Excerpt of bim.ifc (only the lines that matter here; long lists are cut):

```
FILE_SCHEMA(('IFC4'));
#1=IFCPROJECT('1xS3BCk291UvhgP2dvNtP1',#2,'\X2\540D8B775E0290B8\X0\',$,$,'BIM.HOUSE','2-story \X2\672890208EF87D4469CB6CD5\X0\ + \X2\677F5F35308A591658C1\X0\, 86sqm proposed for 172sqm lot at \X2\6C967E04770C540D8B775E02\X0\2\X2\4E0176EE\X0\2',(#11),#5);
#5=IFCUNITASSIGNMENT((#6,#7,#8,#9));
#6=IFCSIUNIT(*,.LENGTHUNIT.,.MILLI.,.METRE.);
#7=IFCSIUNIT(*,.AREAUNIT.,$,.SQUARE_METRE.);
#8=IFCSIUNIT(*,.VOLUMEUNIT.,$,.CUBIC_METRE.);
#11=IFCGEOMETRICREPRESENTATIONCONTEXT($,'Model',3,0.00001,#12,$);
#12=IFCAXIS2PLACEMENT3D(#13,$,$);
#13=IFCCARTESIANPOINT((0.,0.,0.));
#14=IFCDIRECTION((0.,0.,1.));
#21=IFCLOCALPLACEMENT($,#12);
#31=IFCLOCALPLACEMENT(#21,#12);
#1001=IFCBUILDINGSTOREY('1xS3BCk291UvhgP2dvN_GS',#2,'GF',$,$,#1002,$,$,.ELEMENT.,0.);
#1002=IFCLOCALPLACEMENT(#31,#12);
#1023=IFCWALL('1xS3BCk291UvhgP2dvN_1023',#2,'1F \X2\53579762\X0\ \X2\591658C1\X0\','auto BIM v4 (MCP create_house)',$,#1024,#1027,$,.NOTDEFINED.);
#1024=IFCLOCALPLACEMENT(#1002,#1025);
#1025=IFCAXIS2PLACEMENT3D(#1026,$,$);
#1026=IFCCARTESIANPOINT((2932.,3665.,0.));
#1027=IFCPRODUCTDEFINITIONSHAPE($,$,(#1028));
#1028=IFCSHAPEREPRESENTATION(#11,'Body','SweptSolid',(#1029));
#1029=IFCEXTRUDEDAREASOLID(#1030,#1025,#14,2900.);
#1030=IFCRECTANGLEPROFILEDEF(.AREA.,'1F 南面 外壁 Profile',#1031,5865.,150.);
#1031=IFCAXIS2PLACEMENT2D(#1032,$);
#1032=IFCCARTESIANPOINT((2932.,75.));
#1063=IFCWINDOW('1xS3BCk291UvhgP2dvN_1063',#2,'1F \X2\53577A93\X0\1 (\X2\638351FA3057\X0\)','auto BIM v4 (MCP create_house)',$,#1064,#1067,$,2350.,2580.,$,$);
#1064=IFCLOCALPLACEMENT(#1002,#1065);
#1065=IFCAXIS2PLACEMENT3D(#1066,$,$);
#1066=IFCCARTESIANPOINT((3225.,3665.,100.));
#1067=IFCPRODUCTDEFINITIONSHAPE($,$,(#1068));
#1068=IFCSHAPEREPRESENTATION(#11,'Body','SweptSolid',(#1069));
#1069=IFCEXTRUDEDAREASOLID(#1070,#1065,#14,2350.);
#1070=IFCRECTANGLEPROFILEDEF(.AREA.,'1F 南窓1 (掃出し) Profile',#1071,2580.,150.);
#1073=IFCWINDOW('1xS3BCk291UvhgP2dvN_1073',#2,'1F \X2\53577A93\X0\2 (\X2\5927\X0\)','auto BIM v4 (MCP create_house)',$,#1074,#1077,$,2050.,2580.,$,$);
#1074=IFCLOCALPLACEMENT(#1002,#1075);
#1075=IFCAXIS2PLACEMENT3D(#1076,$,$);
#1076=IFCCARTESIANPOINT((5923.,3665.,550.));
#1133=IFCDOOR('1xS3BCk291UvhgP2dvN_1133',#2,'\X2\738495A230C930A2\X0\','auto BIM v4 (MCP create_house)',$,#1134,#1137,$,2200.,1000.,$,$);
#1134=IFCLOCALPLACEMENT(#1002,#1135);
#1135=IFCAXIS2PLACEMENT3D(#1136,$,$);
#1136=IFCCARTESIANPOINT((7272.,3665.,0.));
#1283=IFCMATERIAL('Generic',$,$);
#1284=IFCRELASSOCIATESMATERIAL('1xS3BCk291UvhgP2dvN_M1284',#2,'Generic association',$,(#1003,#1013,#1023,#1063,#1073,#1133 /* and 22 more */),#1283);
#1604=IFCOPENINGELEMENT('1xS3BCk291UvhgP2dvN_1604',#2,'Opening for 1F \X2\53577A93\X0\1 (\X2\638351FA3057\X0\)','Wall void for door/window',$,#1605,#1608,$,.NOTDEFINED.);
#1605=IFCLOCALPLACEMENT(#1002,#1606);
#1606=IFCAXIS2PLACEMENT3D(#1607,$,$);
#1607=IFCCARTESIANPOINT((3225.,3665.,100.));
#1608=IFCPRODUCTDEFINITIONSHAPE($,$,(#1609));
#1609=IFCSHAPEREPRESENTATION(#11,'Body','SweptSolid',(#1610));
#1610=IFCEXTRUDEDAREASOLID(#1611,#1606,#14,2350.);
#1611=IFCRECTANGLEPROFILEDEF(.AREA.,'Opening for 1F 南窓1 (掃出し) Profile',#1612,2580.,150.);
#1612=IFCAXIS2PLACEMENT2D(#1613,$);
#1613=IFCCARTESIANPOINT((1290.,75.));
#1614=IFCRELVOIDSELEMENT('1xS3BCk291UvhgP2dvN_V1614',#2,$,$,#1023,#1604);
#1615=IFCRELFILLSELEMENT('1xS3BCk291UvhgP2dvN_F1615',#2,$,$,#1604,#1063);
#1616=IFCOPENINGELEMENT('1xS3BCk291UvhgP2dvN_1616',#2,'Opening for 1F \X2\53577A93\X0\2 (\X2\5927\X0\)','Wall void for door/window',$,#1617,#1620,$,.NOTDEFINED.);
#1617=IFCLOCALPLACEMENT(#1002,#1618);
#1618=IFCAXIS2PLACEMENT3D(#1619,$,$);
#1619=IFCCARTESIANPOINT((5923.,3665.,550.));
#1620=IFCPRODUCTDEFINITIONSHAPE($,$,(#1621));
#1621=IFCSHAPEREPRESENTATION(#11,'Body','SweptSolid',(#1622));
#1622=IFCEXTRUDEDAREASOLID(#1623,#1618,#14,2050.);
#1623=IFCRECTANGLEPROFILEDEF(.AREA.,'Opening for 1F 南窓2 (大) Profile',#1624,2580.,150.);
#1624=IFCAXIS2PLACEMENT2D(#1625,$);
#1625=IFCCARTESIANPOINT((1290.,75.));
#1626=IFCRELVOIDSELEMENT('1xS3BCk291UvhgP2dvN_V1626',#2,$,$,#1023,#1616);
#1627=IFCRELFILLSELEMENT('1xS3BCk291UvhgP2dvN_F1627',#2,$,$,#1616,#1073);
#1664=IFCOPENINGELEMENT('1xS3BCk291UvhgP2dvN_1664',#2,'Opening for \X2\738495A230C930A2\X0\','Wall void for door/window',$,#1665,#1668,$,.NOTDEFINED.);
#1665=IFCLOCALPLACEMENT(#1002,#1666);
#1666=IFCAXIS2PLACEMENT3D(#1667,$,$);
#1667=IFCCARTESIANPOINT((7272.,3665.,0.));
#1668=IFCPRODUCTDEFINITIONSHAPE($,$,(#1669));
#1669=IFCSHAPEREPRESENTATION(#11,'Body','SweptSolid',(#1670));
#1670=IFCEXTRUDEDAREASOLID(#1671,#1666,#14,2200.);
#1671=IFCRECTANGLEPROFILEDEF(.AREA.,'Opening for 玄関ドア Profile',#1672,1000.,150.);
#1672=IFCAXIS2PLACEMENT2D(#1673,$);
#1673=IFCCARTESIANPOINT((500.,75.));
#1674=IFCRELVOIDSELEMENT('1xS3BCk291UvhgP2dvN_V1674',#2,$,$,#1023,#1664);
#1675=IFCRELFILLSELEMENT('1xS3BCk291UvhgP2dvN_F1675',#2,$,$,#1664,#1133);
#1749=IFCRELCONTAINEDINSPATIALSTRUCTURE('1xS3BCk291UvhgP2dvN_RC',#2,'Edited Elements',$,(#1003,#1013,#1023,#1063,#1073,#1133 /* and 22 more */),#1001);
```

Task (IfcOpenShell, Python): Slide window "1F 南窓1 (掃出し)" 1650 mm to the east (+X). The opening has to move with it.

```python
import ifcopenshell
import ifcopenshell.api.geometry
import ifcopenshell.util.placement
import ifcopenshell.util.unit

model = ifcopenshell.open("bim.ifc")
unit_scale = ifcopenshell.util.unit.calculate_unit_scale(model)

window = model.by_guid("1xS3BCk291UvhgP2dvN_1063")
opening = window.FillsVoids[0].RelatingOpeningElement
wall = opening.VoidsElements[0].RelatingBuildingElement

wall_matrix = ifcopenshell.util.placement.get_local_placement(wall.ObjectPlacement)
shift = wall_matrix[:3, 0] * 1.65 / unit_scale
before = ifcopenshell.util.placement.get_local_placement(window.ObjectPlacement)[:3, 3].copy()

# The window is not placed relative to its opening, so move both.
for product in (opening, window):
    matrix = ifcopenshell.util.placement.get_local_placement(product.ObjectPlacement)
    matrix[:3, 3] += shift
    ifcopenshell.api.geometry.edit_object_placement(model, product=product, matrix=matrix, is_si=False)

after = ifcopenshell.util.placement.get_local_placement(window.ObjectPlacement)[:3, 3]
print("window moved by", (after - before).round(3) + 0.0)

model.write("bim_edited.ifc")
```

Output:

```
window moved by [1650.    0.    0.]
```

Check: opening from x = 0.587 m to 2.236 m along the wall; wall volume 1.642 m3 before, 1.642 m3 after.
